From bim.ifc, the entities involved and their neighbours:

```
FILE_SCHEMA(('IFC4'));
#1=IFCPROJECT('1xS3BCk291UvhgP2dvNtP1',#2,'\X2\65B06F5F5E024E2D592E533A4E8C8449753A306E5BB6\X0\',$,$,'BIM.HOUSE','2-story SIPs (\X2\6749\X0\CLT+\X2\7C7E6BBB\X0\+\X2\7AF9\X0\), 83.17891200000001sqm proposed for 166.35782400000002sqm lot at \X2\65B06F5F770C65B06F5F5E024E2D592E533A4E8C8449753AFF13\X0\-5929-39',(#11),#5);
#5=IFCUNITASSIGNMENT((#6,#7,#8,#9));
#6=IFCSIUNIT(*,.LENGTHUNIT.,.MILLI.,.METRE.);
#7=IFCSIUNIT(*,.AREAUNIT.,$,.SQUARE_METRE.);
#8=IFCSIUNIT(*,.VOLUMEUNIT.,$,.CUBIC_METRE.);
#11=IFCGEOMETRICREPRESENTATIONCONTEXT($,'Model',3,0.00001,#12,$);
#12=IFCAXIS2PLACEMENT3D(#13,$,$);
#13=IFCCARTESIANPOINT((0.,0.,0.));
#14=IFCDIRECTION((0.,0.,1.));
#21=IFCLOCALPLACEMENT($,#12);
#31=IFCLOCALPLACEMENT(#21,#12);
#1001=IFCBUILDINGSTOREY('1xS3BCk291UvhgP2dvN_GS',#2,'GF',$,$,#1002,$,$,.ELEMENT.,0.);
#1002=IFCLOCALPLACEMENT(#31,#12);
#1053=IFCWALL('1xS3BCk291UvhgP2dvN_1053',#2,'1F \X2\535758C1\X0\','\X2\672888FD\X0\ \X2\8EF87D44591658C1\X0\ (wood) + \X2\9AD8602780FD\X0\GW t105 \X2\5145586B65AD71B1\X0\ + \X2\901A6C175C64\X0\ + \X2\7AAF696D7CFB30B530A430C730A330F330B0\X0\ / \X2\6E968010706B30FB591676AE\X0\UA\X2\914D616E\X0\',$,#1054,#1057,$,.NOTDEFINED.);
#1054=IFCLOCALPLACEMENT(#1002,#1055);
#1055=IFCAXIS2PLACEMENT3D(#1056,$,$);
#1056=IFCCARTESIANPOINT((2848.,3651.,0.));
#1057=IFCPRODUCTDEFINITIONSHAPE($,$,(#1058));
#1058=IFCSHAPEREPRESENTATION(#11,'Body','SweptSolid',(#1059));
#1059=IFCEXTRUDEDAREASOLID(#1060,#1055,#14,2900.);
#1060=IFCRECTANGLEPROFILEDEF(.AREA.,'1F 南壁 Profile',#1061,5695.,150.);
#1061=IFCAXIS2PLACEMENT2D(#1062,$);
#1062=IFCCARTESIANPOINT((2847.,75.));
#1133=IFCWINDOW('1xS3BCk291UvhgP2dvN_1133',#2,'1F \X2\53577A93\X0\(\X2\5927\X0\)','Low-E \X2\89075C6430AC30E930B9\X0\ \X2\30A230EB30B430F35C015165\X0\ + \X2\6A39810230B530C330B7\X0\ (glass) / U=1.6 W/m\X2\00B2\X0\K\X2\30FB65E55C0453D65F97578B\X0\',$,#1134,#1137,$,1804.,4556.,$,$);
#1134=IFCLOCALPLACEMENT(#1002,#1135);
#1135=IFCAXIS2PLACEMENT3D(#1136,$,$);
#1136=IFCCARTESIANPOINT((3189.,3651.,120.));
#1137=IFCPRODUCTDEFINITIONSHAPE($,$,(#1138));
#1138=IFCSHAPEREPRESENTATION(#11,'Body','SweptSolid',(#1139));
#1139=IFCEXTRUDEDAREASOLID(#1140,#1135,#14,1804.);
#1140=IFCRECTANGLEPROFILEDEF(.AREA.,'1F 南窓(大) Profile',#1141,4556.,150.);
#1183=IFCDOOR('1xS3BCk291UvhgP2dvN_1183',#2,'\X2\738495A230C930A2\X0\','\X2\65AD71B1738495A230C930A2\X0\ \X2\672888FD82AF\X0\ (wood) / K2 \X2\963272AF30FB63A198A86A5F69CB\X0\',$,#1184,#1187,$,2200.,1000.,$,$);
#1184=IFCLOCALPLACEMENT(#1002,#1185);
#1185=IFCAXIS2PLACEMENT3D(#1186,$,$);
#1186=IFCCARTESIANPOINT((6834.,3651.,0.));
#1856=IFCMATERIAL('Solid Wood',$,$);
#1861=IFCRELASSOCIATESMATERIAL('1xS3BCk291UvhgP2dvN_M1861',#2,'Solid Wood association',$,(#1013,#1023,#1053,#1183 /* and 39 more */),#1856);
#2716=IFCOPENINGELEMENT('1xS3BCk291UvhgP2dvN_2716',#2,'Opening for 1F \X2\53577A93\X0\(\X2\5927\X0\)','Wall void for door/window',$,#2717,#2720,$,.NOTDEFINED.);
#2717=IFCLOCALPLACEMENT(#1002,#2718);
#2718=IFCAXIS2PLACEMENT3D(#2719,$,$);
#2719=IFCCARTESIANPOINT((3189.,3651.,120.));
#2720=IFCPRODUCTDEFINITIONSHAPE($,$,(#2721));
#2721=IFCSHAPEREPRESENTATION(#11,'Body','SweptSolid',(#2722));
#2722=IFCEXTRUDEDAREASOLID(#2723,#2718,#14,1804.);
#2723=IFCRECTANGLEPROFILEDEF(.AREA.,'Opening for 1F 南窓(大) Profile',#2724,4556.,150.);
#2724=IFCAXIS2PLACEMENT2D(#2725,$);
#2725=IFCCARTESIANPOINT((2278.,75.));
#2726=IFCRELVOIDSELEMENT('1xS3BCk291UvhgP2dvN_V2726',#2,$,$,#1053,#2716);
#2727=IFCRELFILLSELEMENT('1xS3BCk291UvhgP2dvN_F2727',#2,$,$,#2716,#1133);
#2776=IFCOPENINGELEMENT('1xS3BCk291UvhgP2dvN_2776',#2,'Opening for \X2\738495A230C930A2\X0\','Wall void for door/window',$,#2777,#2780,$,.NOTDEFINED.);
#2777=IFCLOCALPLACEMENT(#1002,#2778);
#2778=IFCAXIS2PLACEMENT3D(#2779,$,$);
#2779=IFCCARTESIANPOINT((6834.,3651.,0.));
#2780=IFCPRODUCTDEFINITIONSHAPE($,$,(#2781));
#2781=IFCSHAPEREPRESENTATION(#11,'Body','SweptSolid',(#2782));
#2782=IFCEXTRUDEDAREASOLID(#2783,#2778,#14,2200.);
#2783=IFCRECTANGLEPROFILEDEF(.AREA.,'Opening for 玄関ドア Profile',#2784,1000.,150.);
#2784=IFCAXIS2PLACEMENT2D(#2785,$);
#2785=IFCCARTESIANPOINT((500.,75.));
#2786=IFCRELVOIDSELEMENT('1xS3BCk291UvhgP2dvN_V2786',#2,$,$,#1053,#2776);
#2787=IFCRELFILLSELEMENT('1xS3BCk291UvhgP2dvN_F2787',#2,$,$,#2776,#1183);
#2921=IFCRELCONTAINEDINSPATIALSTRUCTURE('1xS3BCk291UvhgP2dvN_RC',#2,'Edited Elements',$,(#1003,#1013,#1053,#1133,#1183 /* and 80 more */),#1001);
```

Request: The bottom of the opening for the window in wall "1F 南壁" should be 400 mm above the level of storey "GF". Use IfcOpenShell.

```python
import numpy as np
import ifcopenshell
import ifcopenshell.api.geometry
import ifcopenshell.geom
import ifcopenshell.util.element
import ifcopenshell.util.placement
import ifcopenshell.util.shape
import ifcopenshell.util.unit

model = ifcopenshell.open("bim.ifc")
unit_scale = ifcopenshell.util.unit.calculate_unit_scale(model)

window = model.by_guid("1xS3BCk291UvhgP2dvN_1133")
opening = window.FillsVoids[0].RelatingOpeningElement
storey = ifcopenshell.util.element.get_container(window, ifc_class="IfcBuildingStorey")
level = ifcopenshell.util.placement.get_local_placement(storey.ObjectPlacement)[2, 3]

# The opening's origin need not be at the sill, so measure its lowest point.
shape = ifcopenshell.geom.create_shape(ifcopenshell.geom.settings(), opening)
bottom = ifcopenshell.util.shape.get_shape_bottom_elevation(shape, shape.geometry) / unit_scale
dz = level + 400.0 - bottom

shift = np.array([0.0, 0.0, dz])
# The window is not placed relative to its opening, so move both.
for product in (opening, window):
    matrix = ifcopenshell.util.placement.get_local_placement(product.ObjectPlacement)
    matrix[:3, 3] += shift
    ifcopenshell.api.geometry.edit_object_placement(model, product=product, matrix=matrix, is_si=False)

print(f"moved by {dz * unit_scale:+.3f} m")

model.write("bim_rev.ifc")
```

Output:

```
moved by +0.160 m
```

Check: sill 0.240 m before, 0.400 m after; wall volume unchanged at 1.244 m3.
